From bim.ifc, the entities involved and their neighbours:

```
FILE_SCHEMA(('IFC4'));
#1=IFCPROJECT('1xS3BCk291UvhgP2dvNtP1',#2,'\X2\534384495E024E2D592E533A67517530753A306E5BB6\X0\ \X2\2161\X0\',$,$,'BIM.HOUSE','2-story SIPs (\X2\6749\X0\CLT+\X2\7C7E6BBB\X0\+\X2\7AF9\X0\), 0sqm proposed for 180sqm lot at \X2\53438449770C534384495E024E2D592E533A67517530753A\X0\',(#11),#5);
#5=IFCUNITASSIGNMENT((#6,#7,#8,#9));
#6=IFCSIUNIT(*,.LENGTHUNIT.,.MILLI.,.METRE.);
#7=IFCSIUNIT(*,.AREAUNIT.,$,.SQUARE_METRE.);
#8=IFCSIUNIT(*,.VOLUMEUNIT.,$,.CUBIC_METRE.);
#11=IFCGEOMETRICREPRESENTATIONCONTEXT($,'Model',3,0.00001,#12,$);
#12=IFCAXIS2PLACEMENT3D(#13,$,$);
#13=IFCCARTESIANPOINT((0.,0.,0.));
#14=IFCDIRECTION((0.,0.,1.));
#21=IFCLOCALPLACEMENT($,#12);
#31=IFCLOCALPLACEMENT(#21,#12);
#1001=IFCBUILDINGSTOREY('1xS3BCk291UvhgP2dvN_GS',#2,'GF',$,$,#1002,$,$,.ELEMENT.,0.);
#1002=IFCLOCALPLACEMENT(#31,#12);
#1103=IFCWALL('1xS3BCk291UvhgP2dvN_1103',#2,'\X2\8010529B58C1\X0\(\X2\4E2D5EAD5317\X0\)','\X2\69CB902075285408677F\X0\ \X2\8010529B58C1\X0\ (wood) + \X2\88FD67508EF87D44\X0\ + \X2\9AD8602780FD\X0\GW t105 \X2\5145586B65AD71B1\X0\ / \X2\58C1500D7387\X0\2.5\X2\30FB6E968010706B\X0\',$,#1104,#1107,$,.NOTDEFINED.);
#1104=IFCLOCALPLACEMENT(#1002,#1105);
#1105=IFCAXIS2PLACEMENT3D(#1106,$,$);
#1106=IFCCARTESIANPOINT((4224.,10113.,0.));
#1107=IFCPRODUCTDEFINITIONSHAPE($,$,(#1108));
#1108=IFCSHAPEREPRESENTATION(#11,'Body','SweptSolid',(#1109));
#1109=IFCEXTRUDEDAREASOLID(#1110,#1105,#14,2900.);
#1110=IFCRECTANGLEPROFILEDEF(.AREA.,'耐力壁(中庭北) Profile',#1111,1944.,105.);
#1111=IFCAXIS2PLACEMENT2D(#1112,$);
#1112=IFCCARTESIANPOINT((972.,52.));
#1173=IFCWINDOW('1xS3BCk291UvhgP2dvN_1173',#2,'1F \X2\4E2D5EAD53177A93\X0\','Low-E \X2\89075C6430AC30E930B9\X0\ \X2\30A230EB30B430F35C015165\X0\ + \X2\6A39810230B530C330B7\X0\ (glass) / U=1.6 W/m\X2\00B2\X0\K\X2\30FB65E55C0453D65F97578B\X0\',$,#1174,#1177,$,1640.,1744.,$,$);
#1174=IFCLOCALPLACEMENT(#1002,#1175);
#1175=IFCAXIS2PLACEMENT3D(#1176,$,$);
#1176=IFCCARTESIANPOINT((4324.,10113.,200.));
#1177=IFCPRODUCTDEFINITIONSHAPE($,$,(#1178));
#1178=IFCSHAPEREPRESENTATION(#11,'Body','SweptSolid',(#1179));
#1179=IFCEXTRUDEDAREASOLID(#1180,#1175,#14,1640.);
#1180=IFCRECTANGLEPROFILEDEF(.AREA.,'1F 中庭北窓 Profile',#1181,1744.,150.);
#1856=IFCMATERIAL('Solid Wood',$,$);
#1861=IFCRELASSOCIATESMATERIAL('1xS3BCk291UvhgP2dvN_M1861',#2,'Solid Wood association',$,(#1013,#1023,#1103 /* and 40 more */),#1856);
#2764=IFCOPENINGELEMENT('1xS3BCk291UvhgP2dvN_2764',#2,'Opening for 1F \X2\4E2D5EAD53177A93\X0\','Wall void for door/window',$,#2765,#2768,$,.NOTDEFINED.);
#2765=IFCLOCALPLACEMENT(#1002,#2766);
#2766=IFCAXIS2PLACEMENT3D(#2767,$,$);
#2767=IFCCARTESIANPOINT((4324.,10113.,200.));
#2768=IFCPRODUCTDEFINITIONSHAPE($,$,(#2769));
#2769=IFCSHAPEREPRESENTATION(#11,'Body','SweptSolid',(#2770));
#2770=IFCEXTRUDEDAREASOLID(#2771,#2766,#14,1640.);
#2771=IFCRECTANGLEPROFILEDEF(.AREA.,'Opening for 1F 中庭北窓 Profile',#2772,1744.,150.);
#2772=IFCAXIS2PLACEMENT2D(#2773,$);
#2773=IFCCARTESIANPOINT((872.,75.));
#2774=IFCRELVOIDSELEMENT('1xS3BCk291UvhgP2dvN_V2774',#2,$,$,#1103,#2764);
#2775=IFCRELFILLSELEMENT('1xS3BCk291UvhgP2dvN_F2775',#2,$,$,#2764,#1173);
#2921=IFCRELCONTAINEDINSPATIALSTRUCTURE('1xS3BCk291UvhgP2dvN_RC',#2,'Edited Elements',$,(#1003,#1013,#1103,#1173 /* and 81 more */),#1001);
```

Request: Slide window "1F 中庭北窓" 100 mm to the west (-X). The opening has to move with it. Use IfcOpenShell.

```python
import ifcopenshell
import ifcopenshell.api.geometry
import ifcopenshell.util.placement
import ifcopenshell.util.unit

model = ifcopenshell.open("bim.ifc")
unit_scale = ifcopenshell.util.unit.calculate_unit_scale(model)

window = model.by_guid("1xS3BCk291UvhgP2dvN_1173")
opening = window.FillsVoids[0].RelatingOpeningElement
wall = opening.VoidsElements[0].RelatingBuildingElement

wall_matrix = ifcopenshell.util.placement.get_local_placement(wall.ObjectPlacement)
shift = wall_matrix[:3, 0] * -0.1 / unit_scale
before = ifcopenshell.util.placement.get_local_placement(window.ObjectPlacement)[:3, 3].copy()

# The window is not placed relative to its opening, so move both.
for product in (opening, window):
    matrix = ifcopenshell.util.placement.get_local_placement(product.ObjectPlacement)
    matrix[:3, 3] += shift
    ifcopenshell.api.geometry.edit_object_placement(model, product=product, matrix=matrix, is_si=False)

after = ifcopenshell.util.placement.get_local_placement(window.ObjectPlacement)[:3, 3]
print("window moved by", (after - before).round(3) + 0.0)

model.write("bim_rev.ifc")
```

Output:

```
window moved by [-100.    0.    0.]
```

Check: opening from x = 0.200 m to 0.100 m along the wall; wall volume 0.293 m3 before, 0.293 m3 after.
